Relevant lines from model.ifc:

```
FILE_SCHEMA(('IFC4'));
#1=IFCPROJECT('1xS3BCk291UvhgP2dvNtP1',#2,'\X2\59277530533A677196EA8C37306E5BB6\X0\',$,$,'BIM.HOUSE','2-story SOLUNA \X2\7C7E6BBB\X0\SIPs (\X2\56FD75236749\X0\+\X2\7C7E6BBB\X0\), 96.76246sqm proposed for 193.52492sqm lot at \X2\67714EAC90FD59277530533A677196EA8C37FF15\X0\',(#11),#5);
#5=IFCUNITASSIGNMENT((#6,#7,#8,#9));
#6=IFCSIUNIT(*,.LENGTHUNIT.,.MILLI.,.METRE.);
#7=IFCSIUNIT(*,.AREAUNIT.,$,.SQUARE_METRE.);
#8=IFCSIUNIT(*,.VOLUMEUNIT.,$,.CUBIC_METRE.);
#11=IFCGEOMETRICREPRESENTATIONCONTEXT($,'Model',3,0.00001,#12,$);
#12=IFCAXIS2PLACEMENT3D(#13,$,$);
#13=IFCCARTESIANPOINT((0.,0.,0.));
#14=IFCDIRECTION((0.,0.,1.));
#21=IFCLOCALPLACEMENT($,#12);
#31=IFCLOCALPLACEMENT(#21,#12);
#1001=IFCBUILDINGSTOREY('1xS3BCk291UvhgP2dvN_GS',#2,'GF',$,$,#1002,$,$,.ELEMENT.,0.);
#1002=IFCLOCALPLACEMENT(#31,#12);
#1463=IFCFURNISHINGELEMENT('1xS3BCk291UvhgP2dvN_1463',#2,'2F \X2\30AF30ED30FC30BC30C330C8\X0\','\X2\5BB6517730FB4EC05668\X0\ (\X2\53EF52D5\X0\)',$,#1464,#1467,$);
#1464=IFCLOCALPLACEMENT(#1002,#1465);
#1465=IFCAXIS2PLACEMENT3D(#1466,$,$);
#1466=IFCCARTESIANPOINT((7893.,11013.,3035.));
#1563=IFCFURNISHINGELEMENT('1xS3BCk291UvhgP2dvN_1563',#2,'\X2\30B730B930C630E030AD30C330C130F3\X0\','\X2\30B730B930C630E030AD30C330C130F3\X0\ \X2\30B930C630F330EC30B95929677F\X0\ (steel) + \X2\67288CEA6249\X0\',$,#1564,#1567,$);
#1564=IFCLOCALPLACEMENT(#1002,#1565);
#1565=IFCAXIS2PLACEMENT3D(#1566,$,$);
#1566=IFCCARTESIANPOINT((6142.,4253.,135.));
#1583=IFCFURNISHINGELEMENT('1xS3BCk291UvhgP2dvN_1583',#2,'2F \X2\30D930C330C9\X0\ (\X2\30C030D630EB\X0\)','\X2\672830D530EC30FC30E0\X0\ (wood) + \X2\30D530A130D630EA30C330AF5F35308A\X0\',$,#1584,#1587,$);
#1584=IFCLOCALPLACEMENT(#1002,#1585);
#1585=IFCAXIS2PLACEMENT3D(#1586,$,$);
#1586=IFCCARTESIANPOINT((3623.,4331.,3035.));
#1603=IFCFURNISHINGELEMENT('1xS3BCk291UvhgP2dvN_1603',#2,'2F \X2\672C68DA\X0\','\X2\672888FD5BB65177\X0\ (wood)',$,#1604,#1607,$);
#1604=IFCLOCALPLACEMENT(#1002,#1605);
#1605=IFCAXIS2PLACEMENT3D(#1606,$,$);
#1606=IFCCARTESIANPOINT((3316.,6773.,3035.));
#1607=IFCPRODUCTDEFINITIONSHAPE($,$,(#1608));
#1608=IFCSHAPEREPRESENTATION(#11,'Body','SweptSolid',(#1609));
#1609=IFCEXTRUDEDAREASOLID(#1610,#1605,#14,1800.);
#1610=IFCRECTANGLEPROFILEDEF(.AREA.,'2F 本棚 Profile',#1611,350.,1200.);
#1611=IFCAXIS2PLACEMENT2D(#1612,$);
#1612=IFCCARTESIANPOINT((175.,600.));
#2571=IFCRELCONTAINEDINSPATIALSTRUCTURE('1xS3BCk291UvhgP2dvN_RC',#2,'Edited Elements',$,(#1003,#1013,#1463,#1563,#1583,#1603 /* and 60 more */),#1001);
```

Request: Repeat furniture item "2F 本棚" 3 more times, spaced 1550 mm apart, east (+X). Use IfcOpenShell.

```python
import numpy as np
import ifcopenshell
import ifcopenshell.api.geometry
import ifcopenshell.api.root
import ifcopenshell.util.element
import ifcopenshell.util.placement

model = ifcopenshell.open("model.ifc")


def reuse_history(source, copy):
    """copy_class also copies each property set's owner history, people and application; keep the originals."""
    for rel in copy.IsDefinedBy:
        if rel.is_a("IfcRelDefinesByProperties") and (history := rel.RelatingPropertyDefinition.OwnerHistory):
            rel.RelatingPropertyDefinition.OwnerHistory = source.OwnerHistory
            ifcopenshell.util.element.remove_deep2(model, history)


source = model.by_id(1603)
base = ifcopenshell.util.placement.get_local_placement(source.ObjectPlacement)
step = np.array([1.0, 0.0, 0.0]) * 1550.0

for i in range(1, 4):
    copy = ifcopenshell.api.root.copy_class(model, product=source)
    copy.Representation = ifcopenshell.util.element.copy_deep(
        model, source.Representation, exclude=["IfcGeometricRepresentationContext", "IfcRepresentationMap"]
    )
    reuse_history(source, copy)
    matrix = base.copy()
    matrix[:3, 3] += i * step
    print("added at", matrix[:3, 3].round(3) + 0.0)
    ifcopenshell.api.geometry.edit_object_placement(model, product=copy, matrix=matrix, is_si=False)

model.write("model_v2.ifc")
```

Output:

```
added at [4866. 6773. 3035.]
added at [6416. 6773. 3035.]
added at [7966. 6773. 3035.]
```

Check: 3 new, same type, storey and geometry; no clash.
